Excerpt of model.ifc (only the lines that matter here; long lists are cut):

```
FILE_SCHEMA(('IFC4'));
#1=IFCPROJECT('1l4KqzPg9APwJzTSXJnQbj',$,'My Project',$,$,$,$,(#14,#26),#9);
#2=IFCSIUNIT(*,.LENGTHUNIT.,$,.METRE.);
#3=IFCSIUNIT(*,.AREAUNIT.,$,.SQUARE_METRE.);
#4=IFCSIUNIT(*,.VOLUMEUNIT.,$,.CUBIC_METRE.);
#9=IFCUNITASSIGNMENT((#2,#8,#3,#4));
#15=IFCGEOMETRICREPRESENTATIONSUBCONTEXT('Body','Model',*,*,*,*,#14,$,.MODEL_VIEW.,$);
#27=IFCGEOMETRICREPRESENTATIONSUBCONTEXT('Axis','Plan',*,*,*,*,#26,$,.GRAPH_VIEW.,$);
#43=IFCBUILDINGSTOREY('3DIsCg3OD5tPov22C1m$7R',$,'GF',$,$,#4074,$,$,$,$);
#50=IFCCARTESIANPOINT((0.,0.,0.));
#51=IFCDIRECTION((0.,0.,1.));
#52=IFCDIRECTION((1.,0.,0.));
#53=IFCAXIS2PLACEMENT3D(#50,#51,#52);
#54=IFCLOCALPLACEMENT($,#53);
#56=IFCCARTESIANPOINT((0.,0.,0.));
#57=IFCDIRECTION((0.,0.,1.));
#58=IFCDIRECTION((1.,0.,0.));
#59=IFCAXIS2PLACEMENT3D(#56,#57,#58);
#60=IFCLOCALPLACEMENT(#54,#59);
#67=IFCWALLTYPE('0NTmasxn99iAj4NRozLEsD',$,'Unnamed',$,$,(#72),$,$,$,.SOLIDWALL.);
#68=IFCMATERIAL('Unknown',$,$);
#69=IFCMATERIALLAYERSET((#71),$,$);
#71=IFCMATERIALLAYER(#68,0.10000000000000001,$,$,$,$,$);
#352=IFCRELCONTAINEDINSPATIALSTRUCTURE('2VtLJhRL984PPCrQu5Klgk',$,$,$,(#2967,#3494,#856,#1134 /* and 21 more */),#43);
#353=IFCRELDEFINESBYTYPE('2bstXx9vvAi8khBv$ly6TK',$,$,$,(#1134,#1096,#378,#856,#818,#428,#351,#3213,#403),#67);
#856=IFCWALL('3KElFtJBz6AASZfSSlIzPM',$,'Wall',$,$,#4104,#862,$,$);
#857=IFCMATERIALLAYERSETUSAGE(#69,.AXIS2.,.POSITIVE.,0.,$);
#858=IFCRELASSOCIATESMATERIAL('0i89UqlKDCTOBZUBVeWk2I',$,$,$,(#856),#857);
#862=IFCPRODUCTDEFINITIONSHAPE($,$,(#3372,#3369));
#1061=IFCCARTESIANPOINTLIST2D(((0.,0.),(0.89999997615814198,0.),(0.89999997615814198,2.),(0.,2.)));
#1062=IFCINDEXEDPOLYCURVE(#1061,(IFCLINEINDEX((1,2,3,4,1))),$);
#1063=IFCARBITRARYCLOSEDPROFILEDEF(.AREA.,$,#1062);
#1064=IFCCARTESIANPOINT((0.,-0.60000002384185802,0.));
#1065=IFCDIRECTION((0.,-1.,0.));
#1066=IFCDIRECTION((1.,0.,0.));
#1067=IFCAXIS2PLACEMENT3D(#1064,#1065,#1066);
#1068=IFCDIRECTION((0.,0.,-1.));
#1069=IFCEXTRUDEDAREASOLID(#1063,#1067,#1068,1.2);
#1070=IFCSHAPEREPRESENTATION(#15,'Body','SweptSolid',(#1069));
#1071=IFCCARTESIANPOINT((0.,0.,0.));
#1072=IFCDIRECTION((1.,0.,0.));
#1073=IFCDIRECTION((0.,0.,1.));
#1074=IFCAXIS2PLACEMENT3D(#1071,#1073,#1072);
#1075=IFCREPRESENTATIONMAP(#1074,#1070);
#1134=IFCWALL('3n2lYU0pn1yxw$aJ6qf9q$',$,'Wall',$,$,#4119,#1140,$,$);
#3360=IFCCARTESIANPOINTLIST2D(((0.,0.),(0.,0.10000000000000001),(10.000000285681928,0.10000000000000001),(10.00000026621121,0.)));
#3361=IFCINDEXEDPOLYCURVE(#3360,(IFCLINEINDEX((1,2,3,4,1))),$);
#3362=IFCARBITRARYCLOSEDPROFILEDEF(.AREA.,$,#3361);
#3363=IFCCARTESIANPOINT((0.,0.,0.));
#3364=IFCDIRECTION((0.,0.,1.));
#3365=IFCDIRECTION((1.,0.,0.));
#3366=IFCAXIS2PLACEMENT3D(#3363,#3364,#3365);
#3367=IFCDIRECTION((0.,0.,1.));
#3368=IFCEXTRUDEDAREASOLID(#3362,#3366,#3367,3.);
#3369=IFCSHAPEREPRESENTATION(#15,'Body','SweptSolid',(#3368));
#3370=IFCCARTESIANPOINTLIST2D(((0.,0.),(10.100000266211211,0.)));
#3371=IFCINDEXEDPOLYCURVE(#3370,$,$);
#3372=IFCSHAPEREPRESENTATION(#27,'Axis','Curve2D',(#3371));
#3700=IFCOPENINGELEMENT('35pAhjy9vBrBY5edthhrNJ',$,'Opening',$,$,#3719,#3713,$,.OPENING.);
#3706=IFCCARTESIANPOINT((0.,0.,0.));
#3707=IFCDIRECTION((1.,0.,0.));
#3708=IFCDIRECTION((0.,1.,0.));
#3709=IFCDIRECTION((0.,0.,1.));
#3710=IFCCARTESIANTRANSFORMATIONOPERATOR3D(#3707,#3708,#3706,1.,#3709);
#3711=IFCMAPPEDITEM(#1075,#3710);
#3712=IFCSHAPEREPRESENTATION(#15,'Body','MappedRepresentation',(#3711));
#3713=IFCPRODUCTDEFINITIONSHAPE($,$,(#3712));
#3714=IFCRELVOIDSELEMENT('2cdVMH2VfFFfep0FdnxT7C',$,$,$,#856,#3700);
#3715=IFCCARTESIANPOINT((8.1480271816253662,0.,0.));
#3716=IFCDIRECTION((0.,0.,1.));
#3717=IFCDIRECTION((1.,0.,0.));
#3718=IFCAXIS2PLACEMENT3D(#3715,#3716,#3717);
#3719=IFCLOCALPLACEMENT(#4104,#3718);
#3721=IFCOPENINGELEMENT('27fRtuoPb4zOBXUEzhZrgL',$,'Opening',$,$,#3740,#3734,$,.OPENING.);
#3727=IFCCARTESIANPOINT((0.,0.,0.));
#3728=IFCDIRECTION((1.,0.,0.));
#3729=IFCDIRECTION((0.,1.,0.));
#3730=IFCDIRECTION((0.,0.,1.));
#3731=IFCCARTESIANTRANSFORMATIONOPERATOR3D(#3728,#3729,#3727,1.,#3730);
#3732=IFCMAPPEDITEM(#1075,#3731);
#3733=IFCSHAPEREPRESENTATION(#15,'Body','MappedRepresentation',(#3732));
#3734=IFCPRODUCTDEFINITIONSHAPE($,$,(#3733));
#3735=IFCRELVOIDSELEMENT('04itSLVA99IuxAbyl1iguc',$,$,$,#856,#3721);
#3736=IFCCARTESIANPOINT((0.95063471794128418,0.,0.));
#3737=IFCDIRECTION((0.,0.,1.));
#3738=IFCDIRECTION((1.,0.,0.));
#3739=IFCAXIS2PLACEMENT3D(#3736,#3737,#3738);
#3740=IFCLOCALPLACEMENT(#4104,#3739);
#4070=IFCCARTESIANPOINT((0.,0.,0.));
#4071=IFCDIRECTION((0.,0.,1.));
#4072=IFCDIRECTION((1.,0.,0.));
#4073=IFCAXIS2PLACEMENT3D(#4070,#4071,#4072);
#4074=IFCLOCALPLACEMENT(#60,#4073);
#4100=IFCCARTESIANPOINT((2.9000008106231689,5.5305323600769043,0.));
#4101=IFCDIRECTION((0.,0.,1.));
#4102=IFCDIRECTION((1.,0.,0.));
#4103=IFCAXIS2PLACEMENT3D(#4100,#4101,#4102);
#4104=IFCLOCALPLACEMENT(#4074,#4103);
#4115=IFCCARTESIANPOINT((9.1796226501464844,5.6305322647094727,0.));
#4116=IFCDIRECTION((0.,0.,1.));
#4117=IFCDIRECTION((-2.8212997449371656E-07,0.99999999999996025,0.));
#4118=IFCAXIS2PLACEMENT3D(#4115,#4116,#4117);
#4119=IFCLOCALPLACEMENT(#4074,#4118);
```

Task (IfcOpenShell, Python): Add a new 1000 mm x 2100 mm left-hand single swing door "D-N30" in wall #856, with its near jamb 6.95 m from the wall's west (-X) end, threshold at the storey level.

```python
import numpy as np
import ifcopenshell
import ifcopenshell.api.feature
import ifcopenshell.api.geometry
import ifcopenshell.api.root
import ifcopenshell.api.spatial
import ifcopenshell.geom
import ifcopenshell.util.element
import ifcopenshell.util.placement
import ifcopenshell.util.representation
import ifcopenshell.util.shape
import ifcopenshell.util.unit

model = ifcopenshell.open("model.ifc")
unit_scale = ifcopenshell.util.unit.calculate_unit_scale(model)
settings = ifcopenshell.geom.settings()


def volume(element):
    """Net volume in cubic metres, openings subtracted."""
    shape = ifcopenshell.geom.create_shape(settings, element)
    return ifcopenshell.util.shape.get_volume(shape.geometry)


wall = model.by_guid("3KElFtJBz6AASZfSSlIzPM")
storey = ifcopenshell.util.element.get_container(wall, ifc_class="IfcBuildingStorey")
context = ifcopenshell.util.representation.get_context(model, "Model", "Body", "MODEL_VIEW")
before = volume(wall)

width, height, from_end, sill = 1, 2.1, 6.95, 0.0  # metres

# The wall runs along its own X axis, and the end named is its -X end.
wall_shape = ifcopenshell.geom.create_shape(settings, wall)
x, y, z = ifcopenshell.util.shape.get_vertices(wall_shape.geometry).T
start = x.min() + from_end
face, thickness = float(y.min()), float(y.max() - y.min())
wall_matrix = ifcopenshell.util.placement.get_local_placement(wall.ObjectPlacement)
level = ifcopenshell.util.placement.get_local_placement(storey.ObjectPlacement)[2, 3]


def in_wall(x, y):
    """Placement at x, y metres in the wall's axes, at sill height."""
    matrix = wall_matrix.copy()
    matrix[:, 3] = wall_matrix @ np.array([x / unit_scale, y / unit_scale, 0.0, 1.0])
    matrix[2, 3] = level + sill / unit_scale
    return matrix


# Opening: a box that overshoots both wall faces by 50 mm.
opening = ifcopenshell.api.root.create_entity(model, ifc_class="IfcOpeningElement", predefined_type="OPENING")
box = ifcopenshell.api.geometry.add_wall_representation(
    model, context=context, length=width, height=height, thickness=thickness + 0.1
)
ifcopenshell.api.geometry.assign_representation(model, product=opening, representation=box)
ifcopenshell.api.geometry.edit_object_placement(model, product=opening, matrix=in_wall(start, face - 0.05), is_si=False)
ifcopenshell.api.feature.add_feature(model, feature=opening, element=wall)

door = ifcopenshell.api.root.create_entity(model, ifc_class="IfcDoor", name="D-N30", predefined_type="DOOR")
door.OverallWidth, door.OverallHeight = width / unit_scale, height / unit_scale
door.OperationType = "SINGLE_SWING_LEFT"
body = ifcopenshell.api.geometry.add_door_representation(
    model,
    context=context,
    overall_width=door.OverallWidth,
    overall_height=door.OverallHeight,
    operation_type="SINGLE_SWING_LEFT",
    lining_properties={"LiningDepth": thickness / unit_scale, "ThresholdDepth": thickness / unit_scale},
)
ifcopenshell.api.geometry.assign_representation(model, product=door, representation=body)
ifcopenshell.api.spatial.assign_container(model, products=[door], relating_structure=storey)
ifcopenshell.api.feature.add_filling(model, opening=opening, element=door)

# The lining spans the wall, so the door starts at the wall face.
ifcopenshell.api.geometry.edit_object_placement(model, product=door, matrix=in_wall(start, face), is_si=False)

after = volume(wall)

print(f"wall volume {before:.3f} -> {after:.3f} m3")

model.write("model_v2.ifc")
```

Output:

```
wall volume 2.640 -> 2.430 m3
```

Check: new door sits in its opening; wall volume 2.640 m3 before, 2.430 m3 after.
